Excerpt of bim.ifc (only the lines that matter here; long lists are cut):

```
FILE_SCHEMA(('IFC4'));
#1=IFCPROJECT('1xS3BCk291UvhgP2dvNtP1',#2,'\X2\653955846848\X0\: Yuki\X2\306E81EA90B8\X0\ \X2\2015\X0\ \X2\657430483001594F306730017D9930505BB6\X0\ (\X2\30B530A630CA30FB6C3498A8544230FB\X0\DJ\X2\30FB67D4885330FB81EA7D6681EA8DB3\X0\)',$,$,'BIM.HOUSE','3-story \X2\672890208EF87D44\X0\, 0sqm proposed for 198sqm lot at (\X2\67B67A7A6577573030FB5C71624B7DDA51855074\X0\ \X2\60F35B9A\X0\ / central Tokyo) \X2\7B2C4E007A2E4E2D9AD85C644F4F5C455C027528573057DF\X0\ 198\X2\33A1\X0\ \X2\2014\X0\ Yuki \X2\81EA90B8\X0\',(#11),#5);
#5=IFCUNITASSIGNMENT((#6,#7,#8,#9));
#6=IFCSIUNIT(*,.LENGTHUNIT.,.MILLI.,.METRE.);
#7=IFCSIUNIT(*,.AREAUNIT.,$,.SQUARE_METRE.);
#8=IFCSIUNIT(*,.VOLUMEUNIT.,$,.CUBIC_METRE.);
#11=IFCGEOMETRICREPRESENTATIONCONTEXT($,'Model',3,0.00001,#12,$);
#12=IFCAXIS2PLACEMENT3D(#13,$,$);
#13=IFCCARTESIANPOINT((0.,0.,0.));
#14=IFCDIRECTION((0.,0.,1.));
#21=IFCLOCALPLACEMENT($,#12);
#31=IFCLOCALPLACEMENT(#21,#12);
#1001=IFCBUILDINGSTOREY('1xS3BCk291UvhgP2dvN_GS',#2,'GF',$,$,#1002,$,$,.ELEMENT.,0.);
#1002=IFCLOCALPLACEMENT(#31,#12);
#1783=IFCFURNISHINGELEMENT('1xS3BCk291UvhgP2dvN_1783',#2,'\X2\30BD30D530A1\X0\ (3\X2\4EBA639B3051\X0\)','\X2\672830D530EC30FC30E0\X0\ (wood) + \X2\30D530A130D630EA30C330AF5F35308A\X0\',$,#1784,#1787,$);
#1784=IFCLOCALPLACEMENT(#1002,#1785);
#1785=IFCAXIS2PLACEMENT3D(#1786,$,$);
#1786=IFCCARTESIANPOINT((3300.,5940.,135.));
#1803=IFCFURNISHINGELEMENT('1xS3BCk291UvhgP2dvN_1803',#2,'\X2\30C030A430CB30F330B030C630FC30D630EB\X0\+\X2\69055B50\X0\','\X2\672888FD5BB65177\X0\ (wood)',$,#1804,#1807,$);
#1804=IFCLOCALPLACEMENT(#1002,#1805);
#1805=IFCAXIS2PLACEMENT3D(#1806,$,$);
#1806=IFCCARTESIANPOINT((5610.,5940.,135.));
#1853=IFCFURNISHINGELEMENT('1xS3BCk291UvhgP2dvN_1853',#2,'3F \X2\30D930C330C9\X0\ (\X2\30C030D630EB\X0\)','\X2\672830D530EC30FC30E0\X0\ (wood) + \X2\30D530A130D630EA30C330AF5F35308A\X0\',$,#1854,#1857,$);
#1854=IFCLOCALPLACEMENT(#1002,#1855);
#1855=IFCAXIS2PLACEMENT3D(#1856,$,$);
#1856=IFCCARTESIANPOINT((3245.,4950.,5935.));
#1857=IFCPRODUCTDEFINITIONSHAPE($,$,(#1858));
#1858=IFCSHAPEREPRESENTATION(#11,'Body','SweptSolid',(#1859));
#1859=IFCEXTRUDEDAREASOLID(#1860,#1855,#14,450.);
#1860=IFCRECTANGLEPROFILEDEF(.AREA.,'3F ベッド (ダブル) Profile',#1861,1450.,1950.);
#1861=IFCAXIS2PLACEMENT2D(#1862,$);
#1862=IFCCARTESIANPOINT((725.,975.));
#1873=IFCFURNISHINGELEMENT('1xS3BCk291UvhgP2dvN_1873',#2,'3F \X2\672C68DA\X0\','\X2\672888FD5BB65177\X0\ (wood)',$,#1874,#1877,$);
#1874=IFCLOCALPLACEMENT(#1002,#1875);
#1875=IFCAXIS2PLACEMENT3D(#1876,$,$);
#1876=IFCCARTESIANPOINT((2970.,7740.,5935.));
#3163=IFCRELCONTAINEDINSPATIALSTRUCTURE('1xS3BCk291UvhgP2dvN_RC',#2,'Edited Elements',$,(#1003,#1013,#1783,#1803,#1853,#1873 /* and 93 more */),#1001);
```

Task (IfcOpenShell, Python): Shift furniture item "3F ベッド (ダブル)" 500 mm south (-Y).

```python
import ifcopenshell
import ifcopenshell.api.geometry
import ifcopenshell.util.placement
import ifcopenshell.util.unit

model = ifcopenshell.open("bim.ifc")
unit_scale = ifcopenshell.util.unit.calculate_unit_scale(model)

item = model.by_guid("1xS3BCk291UvhgP2dvN_1853")
matrix = ifcopenshell.util.placement.get_local_placement(item.ObjectPlacement)
matrix[1, 3] -= 0.5 / unit_scale
ifcopenshell.api.geometry.edit_object_placement(model, product=item, matrix=matrix, is_si=False)

print(ifcopenshell.util.placement.get_local_placement(item.ObjectPlacement).round(3) + 0.0)

model.write("bim_edited.ifc")
```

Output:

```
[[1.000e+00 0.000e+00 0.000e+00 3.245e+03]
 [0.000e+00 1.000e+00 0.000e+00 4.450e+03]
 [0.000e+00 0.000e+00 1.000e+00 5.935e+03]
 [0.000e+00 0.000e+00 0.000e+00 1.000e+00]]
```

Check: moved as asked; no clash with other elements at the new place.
